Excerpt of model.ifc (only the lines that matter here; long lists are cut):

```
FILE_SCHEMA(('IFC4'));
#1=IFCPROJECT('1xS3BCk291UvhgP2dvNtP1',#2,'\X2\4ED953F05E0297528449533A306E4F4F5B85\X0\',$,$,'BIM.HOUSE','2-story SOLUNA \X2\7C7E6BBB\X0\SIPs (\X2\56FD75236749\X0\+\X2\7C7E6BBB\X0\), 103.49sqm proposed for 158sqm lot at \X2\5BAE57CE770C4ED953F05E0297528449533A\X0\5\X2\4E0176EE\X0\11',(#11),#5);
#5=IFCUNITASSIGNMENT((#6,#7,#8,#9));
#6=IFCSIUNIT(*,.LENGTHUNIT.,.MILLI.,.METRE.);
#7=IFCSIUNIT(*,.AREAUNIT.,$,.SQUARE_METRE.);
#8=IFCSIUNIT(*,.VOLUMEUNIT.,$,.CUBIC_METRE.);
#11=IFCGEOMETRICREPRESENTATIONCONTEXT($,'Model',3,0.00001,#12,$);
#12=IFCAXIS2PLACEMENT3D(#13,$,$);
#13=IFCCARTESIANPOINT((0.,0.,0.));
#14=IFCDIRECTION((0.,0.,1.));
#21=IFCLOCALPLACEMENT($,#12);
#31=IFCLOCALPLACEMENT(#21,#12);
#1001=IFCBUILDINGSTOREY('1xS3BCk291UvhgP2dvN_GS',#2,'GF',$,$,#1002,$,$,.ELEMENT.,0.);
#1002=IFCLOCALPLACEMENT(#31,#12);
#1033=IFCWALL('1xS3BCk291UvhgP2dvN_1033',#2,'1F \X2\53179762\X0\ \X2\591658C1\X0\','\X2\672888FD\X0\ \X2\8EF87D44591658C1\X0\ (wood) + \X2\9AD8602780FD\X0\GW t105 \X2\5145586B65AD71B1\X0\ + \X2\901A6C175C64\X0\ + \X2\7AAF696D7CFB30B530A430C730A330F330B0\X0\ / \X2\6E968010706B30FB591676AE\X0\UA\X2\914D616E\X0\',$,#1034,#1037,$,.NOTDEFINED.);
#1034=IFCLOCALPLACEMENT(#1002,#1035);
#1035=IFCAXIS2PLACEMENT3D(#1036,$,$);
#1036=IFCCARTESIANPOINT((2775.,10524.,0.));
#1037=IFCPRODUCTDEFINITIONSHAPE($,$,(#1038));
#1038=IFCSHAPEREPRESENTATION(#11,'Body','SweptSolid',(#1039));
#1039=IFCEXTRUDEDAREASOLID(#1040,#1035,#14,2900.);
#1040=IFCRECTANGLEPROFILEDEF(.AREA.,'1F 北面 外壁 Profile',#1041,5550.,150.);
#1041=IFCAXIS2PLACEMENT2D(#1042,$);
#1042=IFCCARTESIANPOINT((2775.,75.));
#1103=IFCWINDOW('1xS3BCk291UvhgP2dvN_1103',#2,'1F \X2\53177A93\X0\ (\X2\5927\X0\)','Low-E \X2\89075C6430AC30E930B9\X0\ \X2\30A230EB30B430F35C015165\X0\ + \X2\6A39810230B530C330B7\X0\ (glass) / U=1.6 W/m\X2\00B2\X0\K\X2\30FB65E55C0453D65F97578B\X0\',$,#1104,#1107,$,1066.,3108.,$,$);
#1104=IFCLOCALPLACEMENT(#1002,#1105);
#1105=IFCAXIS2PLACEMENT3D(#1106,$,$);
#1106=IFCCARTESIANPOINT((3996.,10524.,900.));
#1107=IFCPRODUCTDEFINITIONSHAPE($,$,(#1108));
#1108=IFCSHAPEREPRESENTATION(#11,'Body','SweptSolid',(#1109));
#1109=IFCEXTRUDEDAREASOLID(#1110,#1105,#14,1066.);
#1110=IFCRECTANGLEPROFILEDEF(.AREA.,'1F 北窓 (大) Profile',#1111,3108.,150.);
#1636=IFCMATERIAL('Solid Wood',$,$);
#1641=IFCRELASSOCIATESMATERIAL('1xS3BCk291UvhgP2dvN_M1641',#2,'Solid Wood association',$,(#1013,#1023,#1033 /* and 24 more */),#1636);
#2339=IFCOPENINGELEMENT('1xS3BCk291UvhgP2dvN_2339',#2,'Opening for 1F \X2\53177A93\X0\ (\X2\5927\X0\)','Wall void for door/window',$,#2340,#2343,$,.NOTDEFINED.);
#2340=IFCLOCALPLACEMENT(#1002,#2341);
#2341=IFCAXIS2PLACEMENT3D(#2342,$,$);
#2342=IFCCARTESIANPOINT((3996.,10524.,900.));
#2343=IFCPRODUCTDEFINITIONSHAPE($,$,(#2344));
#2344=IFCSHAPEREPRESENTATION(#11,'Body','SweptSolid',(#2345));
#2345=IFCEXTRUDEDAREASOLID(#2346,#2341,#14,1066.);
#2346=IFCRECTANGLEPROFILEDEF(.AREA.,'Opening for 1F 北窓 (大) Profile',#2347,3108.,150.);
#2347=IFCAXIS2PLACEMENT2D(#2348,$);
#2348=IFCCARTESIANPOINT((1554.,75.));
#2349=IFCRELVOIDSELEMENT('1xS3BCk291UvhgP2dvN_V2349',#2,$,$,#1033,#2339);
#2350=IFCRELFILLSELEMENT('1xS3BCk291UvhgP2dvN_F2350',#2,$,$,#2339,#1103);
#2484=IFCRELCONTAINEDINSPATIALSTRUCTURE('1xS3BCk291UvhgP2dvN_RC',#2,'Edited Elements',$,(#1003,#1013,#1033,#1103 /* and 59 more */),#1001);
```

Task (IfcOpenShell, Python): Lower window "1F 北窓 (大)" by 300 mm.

```python
import numpy as np
import ifcopenshell
import ifcopenshell.api.geometry
import ifcopenshell.util.placement
import ifcopenshell.util.unit

model = ifcopenshell.open("model.ifc")
unit_scale = ifcopenshell.util.unit.calculate_unit_scale(model)

window = model.by_guid("1xS3BCk291UvhgP2dvN_1103")
opening = window.FillsVoids[0].RelatingOpeningElement
dz = -300.0

shift = np.array([0.0, 0.0, dz])
# The window is not placed relative to its opening, so move both.
for product in (opening, window):
    matrix = ifcopenshell.util.placement.get_local_placement(product.ObjectPlacement)
    matrix[:3, 3] += shift
    ifcopenshell.api.geometry.edit_object_placement(model, product=product, matrix=matrix, is_si=False)

print(f"moved by {dz * unit_scale:+.3f} m")

model.write("model_updated.ifc")
```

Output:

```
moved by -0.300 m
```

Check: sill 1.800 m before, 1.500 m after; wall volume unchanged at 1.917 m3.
